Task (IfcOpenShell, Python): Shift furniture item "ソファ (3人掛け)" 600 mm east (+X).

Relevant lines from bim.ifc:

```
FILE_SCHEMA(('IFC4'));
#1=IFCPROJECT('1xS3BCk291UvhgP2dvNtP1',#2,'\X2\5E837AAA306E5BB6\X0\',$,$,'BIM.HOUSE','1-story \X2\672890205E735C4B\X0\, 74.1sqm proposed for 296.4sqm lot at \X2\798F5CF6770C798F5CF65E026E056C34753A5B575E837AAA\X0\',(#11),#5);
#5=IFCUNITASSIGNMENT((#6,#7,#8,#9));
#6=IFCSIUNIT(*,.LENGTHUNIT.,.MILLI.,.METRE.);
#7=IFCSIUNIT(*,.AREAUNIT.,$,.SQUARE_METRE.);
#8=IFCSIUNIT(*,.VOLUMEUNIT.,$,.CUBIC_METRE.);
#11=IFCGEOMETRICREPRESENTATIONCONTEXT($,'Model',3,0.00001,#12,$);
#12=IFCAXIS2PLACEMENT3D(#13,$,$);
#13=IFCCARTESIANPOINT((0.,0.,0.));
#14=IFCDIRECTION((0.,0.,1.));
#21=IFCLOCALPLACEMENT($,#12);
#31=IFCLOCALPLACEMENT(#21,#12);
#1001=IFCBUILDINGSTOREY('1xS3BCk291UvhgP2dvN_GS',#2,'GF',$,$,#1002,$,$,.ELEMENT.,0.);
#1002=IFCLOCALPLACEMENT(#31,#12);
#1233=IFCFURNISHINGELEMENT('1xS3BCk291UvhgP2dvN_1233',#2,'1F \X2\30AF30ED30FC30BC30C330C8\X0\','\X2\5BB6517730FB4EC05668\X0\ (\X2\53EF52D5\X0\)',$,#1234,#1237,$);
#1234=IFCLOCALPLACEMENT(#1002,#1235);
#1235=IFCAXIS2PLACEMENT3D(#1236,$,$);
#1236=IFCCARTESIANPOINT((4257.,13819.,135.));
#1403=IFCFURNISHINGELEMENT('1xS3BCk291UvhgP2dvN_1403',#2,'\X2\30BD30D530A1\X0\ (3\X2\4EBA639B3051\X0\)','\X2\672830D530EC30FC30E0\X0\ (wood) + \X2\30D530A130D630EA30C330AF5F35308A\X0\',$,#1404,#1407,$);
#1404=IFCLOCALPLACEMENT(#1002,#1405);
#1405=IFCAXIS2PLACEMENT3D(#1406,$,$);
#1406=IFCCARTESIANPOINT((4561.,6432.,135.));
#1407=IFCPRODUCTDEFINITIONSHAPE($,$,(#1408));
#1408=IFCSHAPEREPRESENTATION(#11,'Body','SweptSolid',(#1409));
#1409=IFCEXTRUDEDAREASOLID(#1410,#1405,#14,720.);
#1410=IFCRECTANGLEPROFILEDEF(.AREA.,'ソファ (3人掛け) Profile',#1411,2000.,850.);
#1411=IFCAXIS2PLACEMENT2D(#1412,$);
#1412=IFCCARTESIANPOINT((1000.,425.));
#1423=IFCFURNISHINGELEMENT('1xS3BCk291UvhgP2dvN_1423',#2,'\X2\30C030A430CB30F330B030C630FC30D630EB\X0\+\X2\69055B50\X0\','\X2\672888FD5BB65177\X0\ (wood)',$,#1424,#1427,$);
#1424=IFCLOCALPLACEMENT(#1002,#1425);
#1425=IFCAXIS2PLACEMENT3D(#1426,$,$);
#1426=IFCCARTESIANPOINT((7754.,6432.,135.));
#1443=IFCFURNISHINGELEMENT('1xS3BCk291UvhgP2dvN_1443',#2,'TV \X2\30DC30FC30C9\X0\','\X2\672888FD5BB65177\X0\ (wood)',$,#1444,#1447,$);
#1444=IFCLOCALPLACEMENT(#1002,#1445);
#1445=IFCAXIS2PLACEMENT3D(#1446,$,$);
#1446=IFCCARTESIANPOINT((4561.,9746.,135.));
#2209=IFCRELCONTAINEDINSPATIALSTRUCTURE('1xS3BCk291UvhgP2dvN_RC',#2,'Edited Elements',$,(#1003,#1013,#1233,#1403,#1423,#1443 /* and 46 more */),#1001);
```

```python
import ifcopenshell
import ifcopenshell.api.geometry
import ifcopenshell.util.placement
import ifcopenshell.util.unit

model = ifcopenshell.open("bim.ifc")
unit_scale = ifcopenshell.util.unit.calculate_unit_scale(model)

item = model.by_guid("1xS3BCk291UvhgP2dvN_1403")
matrix = ifcopenshell.util.placement.get_local_placement(item.ObjectPlacement)
matrix[0, 3] += 0.6 / unit_scale
ifcopenshell.api.geometry.edit_object_placement(model, product=item, matrix=matrix, is_si=False)

print(ifcopenshell.util.placement.get_local_placement(item.ObjectPlacement).round(3) + 0.0)

model.write("bim_rev.ifc")
```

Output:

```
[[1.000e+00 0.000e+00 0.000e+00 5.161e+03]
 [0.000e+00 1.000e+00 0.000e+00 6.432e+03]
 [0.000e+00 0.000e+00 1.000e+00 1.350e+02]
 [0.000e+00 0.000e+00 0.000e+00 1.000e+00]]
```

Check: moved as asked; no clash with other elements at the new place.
